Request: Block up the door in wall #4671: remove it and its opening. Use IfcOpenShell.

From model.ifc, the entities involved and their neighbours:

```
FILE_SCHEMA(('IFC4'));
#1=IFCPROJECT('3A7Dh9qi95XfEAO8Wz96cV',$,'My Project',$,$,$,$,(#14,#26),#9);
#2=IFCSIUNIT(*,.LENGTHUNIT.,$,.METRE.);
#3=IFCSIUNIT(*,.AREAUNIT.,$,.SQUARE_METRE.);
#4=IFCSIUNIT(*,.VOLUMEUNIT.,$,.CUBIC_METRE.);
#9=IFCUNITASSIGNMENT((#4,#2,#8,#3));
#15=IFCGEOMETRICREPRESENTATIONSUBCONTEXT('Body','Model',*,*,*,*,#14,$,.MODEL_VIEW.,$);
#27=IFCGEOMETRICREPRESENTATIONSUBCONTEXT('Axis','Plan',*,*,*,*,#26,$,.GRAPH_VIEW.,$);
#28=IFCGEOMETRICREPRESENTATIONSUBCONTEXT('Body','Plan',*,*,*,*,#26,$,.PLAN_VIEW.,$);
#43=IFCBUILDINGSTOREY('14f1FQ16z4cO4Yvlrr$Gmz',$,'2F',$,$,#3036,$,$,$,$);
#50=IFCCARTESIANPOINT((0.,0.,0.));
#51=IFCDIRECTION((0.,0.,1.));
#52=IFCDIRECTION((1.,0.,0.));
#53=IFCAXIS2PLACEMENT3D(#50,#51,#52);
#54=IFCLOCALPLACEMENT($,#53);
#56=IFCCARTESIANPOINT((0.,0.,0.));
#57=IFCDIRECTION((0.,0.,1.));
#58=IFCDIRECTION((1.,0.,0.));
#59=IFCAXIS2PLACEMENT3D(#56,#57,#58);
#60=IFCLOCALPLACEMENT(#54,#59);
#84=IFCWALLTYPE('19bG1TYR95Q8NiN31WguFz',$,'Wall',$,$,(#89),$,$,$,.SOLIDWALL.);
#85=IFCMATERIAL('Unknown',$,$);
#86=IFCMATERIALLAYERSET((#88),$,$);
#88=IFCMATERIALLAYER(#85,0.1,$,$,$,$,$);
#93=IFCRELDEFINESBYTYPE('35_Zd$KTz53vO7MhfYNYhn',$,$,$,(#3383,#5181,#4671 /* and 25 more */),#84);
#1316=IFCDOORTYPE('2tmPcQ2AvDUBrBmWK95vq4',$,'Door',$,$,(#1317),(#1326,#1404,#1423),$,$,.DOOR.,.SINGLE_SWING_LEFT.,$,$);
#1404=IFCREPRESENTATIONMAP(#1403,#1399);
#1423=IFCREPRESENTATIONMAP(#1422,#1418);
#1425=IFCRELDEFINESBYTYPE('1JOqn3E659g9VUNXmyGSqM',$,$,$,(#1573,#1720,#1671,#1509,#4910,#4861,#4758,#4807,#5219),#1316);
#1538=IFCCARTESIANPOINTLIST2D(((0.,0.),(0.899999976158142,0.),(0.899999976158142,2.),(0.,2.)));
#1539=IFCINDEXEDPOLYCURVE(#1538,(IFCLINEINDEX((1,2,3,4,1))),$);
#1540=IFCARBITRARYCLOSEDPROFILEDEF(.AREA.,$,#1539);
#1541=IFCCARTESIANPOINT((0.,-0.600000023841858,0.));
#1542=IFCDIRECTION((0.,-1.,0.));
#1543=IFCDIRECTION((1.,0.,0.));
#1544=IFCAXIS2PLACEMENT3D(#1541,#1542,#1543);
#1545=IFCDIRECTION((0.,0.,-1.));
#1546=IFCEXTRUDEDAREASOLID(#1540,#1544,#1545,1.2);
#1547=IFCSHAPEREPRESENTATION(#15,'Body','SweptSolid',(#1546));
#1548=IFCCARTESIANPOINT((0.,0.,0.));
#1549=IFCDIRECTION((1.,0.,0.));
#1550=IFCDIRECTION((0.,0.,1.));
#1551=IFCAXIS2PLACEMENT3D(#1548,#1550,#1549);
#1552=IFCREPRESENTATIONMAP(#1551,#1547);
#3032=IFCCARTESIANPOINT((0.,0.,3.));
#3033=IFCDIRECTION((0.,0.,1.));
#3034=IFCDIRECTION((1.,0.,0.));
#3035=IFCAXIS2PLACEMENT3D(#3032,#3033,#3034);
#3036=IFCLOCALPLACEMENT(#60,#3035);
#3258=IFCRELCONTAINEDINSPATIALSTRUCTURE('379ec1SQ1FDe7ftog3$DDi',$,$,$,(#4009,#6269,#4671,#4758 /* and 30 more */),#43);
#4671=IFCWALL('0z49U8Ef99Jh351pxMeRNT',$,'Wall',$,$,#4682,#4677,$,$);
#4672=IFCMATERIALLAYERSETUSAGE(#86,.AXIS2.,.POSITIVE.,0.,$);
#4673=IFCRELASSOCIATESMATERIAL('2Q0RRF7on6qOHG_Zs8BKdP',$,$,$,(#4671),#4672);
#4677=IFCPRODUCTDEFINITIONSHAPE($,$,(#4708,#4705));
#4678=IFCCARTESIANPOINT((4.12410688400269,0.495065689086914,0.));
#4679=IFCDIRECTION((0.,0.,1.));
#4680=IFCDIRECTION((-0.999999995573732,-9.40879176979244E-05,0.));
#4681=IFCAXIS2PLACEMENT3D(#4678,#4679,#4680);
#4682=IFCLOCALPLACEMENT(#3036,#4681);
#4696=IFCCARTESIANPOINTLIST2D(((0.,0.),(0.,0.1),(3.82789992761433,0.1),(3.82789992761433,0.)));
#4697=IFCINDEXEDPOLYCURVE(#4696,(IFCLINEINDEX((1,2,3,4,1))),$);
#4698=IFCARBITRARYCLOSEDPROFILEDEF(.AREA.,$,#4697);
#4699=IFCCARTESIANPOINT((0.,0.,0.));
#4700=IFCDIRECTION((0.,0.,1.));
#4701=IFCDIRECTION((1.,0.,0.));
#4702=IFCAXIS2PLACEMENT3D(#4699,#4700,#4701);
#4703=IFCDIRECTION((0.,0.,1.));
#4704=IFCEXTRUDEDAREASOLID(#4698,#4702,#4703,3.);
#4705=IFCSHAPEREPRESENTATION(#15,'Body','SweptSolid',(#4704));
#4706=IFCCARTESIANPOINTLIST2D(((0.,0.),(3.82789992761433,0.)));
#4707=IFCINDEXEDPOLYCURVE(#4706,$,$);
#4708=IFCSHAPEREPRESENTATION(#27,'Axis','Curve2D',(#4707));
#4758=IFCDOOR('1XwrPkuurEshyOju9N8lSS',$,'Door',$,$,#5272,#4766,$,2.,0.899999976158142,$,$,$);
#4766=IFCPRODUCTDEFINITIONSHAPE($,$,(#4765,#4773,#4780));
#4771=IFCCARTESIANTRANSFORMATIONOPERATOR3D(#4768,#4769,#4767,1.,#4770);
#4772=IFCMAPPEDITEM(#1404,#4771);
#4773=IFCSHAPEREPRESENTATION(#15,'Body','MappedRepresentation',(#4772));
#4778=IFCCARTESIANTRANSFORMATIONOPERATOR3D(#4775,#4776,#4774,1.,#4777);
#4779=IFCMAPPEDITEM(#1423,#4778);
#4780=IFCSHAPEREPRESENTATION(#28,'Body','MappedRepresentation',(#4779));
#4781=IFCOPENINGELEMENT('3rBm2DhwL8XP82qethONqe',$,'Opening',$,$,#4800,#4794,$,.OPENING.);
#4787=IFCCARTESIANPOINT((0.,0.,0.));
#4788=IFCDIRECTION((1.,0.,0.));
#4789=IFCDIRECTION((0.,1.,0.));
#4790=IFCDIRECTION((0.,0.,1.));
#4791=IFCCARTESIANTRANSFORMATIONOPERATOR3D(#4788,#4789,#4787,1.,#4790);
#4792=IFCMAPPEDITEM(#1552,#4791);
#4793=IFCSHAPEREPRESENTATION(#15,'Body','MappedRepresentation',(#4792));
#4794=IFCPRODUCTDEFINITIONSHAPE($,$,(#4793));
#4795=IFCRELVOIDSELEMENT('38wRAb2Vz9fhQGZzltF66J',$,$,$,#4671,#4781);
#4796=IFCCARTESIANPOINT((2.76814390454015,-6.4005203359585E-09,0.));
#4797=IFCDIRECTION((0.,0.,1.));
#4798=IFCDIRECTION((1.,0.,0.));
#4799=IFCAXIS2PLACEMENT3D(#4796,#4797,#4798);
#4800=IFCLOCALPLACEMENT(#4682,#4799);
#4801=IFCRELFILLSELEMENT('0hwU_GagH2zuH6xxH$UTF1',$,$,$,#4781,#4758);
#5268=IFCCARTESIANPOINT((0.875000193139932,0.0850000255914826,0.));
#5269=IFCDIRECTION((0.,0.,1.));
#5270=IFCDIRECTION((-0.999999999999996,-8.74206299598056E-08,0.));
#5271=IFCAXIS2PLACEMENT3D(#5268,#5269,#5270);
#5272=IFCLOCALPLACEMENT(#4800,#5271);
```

```python
import ifcopenshell
import ifcopenshell.api.feature
import ifcopenshell.api.root
import ifcopenshell.geom
import ifcopenshell.util.shape

model = ifcopenshell.open("model.ifc")
settings = ifcopenshell.geom.settings()


def volume(element):
    """Net volume in cubic metres, openings subtracted."""
    shape = ifcopenshell.geom.create_shape(settings, element)
    return ifcopenshell.util.shape.get_volume(shape.geometry)


door = model.by_id(4758)
opening = door.FillsVoids[0].RelatingOpeningElement
wall = opening.VoidsElements[0].RelatingBuildingElement
before = volume(wall)

ifcopenshell.api.root.remove_product(model, product=door)
ifcopenshell.api.feature.remove_feature(model, feature=opening)

after = volume(wall)

print(f"wall volume {before:.3f} -> {after:.3f} m3")

model.write("model-out.ifc")
```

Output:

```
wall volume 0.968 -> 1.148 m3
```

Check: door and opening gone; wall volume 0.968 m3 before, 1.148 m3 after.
